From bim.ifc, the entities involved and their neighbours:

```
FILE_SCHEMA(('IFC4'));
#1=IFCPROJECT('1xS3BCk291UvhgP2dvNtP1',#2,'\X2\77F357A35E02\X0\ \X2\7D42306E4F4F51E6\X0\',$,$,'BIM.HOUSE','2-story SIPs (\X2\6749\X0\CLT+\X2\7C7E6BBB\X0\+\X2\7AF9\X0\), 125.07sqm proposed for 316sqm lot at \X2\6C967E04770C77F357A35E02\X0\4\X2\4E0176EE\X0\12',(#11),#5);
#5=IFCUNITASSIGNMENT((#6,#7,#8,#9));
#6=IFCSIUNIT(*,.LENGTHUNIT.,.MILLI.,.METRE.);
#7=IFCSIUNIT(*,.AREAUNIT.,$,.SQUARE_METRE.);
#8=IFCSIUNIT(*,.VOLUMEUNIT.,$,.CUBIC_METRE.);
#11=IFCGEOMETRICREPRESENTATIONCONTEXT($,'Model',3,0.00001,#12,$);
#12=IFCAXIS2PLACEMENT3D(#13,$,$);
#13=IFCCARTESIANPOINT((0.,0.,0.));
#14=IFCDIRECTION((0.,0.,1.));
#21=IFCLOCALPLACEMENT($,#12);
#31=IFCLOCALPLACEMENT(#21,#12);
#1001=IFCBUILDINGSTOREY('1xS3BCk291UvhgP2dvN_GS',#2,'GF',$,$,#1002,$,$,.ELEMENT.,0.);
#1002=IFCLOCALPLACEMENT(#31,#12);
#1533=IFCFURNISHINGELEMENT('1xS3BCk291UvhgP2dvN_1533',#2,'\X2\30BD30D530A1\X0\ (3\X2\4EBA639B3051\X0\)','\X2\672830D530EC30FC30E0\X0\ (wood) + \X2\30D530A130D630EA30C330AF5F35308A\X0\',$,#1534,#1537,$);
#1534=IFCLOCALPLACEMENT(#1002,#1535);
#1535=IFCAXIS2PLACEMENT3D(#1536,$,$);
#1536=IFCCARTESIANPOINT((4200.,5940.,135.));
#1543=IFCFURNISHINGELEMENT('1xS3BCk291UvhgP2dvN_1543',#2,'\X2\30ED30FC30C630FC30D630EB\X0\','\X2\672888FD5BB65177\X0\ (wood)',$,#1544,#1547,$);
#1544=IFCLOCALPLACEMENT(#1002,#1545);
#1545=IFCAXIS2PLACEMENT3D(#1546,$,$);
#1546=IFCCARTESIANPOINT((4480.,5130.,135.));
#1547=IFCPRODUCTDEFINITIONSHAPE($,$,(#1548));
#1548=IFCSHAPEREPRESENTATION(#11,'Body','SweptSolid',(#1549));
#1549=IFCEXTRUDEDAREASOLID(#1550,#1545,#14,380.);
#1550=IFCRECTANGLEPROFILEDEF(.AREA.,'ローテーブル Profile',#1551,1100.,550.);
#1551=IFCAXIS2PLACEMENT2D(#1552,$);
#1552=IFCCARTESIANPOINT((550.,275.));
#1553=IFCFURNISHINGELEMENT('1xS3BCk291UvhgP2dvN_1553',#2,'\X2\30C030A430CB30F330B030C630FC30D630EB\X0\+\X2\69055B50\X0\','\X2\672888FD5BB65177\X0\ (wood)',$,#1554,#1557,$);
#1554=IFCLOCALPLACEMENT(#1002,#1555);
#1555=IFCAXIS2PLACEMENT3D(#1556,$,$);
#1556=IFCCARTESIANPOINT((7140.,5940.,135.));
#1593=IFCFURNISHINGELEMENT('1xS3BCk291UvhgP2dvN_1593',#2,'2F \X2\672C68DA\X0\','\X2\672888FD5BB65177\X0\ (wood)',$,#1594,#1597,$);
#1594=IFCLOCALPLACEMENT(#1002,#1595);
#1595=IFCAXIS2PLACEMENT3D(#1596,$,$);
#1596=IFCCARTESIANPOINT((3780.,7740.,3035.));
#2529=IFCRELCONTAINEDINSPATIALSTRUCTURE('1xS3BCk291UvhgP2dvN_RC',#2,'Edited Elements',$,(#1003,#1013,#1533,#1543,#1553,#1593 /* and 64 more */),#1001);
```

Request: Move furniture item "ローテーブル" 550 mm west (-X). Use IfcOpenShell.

```python
import ifcopenshell
import ifcopenshell.api.geometry
import ifcopenshell.util.placement
import ifcopenshell.util.unit

model = ifcopenshell.open("bim.ifc")
unit_scale = ifcopenshell.util.unit.calculate_unit_scale(model)

item = model.by_guid("1xS3BCk291UvhgP2dvN_1543")
matrix = ifcopenshell.util.placement.get_local_placement(item.ObjectPlacement)
matrix[0, 3] -= 0.55 / unit_scale
ifcopenshell.api.geometry.edit_object_placement(model, product=item, matrix=matrix, is_si=False)

print(ifcopenshell.util.placement.get_local_placement(item.ObjectPlacement).round(3) + 0.0)

model.write("bim_edited.ifc")
```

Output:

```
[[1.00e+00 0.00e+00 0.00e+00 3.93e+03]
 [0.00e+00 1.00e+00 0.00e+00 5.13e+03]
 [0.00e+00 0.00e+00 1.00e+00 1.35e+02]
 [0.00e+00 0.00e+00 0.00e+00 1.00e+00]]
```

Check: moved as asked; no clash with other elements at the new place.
